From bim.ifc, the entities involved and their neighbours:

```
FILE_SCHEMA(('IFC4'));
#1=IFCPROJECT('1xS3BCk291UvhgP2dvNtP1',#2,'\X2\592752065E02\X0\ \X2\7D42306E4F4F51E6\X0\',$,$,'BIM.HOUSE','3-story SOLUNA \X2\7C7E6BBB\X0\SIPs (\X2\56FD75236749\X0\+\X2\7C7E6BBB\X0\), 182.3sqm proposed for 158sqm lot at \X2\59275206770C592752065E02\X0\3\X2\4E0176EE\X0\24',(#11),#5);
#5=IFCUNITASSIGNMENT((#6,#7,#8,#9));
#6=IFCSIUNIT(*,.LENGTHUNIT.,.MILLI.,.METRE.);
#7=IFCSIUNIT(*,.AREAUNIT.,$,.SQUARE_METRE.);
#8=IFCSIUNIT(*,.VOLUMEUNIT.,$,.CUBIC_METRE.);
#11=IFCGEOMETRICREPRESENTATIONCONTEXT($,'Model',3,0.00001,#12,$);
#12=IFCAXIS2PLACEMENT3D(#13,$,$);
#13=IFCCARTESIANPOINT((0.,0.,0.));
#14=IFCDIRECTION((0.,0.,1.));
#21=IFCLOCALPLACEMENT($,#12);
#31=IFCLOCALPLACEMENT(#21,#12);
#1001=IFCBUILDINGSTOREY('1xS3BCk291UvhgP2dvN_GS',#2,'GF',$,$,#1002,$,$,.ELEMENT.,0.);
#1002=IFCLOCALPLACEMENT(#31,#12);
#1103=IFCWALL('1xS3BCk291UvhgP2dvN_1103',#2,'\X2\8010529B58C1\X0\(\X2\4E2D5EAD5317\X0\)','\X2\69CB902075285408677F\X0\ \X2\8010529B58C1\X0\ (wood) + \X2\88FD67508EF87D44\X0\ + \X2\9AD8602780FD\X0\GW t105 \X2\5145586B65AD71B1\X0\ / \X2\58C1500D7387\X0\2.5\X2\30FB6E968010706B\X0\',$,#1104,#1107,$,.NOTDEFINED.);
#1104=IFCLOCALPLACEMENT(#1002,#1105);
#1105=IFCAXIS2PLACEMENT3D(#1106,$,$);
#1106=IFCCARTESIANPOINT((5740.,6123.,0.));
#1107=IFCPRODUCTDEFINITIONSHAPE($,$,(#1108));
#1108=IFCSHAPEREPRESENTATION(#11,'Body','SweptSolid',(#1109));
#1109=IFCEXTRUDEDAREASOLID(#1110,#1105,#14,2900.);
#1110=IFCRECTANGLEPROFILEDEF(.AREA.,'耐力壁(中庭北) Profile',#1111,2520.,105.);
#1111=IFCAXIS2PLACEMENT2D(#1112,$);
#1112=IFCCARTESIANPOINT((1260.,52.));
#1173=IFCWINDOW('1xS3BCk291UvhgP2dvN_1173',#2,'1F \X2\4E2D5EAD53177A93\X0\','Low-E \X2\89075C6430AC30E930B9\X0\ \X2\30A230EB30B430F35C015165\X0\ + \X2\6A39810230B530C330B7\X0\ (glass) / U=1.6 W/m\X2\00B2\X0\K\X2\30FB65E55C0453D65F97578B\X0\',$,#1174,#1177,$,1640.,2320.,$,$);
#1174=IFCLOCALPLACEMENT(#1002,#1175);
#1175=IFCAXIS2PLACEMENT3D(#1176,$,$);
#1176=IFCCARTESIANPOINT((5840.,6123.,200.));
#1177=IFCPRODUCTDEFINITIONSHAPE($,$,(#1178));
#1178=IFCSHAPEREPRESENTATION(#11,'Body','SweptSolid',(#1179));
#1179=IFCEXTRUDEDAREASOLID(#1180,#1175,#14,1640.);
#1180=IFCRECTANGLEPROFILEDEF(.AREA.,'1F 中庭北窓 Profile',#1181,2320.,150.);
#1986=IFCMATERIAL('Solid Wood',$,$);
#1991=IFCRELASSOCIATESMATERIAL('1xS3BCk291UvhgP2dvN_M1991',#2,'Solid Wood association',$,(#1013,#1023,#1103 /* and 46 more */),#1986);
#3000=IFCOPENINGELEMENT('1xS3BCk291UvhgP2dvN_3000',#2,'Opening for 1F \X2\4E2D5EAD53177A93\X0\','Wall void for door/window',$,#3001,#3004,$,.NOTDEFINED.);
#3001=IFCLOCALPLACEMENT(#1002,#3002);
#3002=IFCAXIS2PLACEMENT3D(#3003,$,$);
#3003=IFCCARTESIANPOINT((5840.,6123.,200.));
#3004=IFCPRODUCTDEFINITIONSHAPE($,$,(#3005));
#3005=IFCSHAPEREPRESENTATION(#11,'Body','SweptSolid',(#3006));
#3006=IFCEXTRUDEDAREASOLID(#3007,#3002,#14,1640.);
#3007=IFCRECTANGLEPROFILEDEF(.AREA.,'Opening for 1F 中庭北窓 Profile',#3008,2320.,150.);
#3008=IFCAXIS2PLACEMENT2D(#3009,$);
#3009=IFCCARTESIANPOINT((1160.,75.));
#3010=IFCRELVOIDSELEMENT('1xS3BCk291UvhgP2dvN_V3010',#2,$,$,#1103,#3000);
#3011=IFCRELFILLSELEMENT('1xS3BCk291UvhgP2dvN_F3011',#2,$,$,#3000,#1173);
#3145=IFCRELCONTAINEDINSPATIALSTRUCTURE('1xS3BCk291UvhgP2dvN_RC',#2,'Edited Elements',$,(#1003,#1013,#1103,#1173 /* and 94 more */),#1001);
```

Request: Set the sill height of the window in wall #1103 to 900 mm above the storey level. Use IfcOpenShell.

```python
import numpy as np
import ifcopenshell
import ifcopenshell.api.geometry
import ifcopenshell.geom
import ifcopenshell.util.element
import ifcopenshell.util.placement
import ifcopenshell.util.shape
import ifcopenshell.util.unit

model = ifcopenshell.open("bim.ifc")
unit_scale = ifcopenshell.util.unit.calculate_unit_scale(model)

window = model.by_guid("1xS3BCk291UvhgP2dvN_1173")
opening = window.FillsVoids[0].RelatingOpeningElement
storey = ifcopenshell.util.element.get_container(window, ifc_class="IfcBuildingStorey")
level = ifcopenshell.util.placement.get_local_placement(storey.ObjectPlacement)[2, 3]

# The opening's origin need not be at the sill, so measure its lowest point.
shape = ifcopenshell.geom.create_shape(ifcopenshell.geom.settings(), opening)
bottom = ifcopenshell.util.shape.get_shape_bottom_elevation(shape, shape.geometry) / unit_scale
dz = level + 900.0 - bottom

shift = np.array([0.0, 0.0, dz])
# The window is not placed relative to its opening, so move both.
for product in (opening, window):
    matrix = ifcopenshell.util.placement.get_local_placement(product.ObjectPlacement)
    matrix[:3, 3] += shift
    ifcopenshell.api.geometry.edit_object_placement(model, product=product, matrix=matrix, is_si=False)

print(f"moved by {dz * unit_scale:+.3f} m")

model.write("bim_rev.ifc")
```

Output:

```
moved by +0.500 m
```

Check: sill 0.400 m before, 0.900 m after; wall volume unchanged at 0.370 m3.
